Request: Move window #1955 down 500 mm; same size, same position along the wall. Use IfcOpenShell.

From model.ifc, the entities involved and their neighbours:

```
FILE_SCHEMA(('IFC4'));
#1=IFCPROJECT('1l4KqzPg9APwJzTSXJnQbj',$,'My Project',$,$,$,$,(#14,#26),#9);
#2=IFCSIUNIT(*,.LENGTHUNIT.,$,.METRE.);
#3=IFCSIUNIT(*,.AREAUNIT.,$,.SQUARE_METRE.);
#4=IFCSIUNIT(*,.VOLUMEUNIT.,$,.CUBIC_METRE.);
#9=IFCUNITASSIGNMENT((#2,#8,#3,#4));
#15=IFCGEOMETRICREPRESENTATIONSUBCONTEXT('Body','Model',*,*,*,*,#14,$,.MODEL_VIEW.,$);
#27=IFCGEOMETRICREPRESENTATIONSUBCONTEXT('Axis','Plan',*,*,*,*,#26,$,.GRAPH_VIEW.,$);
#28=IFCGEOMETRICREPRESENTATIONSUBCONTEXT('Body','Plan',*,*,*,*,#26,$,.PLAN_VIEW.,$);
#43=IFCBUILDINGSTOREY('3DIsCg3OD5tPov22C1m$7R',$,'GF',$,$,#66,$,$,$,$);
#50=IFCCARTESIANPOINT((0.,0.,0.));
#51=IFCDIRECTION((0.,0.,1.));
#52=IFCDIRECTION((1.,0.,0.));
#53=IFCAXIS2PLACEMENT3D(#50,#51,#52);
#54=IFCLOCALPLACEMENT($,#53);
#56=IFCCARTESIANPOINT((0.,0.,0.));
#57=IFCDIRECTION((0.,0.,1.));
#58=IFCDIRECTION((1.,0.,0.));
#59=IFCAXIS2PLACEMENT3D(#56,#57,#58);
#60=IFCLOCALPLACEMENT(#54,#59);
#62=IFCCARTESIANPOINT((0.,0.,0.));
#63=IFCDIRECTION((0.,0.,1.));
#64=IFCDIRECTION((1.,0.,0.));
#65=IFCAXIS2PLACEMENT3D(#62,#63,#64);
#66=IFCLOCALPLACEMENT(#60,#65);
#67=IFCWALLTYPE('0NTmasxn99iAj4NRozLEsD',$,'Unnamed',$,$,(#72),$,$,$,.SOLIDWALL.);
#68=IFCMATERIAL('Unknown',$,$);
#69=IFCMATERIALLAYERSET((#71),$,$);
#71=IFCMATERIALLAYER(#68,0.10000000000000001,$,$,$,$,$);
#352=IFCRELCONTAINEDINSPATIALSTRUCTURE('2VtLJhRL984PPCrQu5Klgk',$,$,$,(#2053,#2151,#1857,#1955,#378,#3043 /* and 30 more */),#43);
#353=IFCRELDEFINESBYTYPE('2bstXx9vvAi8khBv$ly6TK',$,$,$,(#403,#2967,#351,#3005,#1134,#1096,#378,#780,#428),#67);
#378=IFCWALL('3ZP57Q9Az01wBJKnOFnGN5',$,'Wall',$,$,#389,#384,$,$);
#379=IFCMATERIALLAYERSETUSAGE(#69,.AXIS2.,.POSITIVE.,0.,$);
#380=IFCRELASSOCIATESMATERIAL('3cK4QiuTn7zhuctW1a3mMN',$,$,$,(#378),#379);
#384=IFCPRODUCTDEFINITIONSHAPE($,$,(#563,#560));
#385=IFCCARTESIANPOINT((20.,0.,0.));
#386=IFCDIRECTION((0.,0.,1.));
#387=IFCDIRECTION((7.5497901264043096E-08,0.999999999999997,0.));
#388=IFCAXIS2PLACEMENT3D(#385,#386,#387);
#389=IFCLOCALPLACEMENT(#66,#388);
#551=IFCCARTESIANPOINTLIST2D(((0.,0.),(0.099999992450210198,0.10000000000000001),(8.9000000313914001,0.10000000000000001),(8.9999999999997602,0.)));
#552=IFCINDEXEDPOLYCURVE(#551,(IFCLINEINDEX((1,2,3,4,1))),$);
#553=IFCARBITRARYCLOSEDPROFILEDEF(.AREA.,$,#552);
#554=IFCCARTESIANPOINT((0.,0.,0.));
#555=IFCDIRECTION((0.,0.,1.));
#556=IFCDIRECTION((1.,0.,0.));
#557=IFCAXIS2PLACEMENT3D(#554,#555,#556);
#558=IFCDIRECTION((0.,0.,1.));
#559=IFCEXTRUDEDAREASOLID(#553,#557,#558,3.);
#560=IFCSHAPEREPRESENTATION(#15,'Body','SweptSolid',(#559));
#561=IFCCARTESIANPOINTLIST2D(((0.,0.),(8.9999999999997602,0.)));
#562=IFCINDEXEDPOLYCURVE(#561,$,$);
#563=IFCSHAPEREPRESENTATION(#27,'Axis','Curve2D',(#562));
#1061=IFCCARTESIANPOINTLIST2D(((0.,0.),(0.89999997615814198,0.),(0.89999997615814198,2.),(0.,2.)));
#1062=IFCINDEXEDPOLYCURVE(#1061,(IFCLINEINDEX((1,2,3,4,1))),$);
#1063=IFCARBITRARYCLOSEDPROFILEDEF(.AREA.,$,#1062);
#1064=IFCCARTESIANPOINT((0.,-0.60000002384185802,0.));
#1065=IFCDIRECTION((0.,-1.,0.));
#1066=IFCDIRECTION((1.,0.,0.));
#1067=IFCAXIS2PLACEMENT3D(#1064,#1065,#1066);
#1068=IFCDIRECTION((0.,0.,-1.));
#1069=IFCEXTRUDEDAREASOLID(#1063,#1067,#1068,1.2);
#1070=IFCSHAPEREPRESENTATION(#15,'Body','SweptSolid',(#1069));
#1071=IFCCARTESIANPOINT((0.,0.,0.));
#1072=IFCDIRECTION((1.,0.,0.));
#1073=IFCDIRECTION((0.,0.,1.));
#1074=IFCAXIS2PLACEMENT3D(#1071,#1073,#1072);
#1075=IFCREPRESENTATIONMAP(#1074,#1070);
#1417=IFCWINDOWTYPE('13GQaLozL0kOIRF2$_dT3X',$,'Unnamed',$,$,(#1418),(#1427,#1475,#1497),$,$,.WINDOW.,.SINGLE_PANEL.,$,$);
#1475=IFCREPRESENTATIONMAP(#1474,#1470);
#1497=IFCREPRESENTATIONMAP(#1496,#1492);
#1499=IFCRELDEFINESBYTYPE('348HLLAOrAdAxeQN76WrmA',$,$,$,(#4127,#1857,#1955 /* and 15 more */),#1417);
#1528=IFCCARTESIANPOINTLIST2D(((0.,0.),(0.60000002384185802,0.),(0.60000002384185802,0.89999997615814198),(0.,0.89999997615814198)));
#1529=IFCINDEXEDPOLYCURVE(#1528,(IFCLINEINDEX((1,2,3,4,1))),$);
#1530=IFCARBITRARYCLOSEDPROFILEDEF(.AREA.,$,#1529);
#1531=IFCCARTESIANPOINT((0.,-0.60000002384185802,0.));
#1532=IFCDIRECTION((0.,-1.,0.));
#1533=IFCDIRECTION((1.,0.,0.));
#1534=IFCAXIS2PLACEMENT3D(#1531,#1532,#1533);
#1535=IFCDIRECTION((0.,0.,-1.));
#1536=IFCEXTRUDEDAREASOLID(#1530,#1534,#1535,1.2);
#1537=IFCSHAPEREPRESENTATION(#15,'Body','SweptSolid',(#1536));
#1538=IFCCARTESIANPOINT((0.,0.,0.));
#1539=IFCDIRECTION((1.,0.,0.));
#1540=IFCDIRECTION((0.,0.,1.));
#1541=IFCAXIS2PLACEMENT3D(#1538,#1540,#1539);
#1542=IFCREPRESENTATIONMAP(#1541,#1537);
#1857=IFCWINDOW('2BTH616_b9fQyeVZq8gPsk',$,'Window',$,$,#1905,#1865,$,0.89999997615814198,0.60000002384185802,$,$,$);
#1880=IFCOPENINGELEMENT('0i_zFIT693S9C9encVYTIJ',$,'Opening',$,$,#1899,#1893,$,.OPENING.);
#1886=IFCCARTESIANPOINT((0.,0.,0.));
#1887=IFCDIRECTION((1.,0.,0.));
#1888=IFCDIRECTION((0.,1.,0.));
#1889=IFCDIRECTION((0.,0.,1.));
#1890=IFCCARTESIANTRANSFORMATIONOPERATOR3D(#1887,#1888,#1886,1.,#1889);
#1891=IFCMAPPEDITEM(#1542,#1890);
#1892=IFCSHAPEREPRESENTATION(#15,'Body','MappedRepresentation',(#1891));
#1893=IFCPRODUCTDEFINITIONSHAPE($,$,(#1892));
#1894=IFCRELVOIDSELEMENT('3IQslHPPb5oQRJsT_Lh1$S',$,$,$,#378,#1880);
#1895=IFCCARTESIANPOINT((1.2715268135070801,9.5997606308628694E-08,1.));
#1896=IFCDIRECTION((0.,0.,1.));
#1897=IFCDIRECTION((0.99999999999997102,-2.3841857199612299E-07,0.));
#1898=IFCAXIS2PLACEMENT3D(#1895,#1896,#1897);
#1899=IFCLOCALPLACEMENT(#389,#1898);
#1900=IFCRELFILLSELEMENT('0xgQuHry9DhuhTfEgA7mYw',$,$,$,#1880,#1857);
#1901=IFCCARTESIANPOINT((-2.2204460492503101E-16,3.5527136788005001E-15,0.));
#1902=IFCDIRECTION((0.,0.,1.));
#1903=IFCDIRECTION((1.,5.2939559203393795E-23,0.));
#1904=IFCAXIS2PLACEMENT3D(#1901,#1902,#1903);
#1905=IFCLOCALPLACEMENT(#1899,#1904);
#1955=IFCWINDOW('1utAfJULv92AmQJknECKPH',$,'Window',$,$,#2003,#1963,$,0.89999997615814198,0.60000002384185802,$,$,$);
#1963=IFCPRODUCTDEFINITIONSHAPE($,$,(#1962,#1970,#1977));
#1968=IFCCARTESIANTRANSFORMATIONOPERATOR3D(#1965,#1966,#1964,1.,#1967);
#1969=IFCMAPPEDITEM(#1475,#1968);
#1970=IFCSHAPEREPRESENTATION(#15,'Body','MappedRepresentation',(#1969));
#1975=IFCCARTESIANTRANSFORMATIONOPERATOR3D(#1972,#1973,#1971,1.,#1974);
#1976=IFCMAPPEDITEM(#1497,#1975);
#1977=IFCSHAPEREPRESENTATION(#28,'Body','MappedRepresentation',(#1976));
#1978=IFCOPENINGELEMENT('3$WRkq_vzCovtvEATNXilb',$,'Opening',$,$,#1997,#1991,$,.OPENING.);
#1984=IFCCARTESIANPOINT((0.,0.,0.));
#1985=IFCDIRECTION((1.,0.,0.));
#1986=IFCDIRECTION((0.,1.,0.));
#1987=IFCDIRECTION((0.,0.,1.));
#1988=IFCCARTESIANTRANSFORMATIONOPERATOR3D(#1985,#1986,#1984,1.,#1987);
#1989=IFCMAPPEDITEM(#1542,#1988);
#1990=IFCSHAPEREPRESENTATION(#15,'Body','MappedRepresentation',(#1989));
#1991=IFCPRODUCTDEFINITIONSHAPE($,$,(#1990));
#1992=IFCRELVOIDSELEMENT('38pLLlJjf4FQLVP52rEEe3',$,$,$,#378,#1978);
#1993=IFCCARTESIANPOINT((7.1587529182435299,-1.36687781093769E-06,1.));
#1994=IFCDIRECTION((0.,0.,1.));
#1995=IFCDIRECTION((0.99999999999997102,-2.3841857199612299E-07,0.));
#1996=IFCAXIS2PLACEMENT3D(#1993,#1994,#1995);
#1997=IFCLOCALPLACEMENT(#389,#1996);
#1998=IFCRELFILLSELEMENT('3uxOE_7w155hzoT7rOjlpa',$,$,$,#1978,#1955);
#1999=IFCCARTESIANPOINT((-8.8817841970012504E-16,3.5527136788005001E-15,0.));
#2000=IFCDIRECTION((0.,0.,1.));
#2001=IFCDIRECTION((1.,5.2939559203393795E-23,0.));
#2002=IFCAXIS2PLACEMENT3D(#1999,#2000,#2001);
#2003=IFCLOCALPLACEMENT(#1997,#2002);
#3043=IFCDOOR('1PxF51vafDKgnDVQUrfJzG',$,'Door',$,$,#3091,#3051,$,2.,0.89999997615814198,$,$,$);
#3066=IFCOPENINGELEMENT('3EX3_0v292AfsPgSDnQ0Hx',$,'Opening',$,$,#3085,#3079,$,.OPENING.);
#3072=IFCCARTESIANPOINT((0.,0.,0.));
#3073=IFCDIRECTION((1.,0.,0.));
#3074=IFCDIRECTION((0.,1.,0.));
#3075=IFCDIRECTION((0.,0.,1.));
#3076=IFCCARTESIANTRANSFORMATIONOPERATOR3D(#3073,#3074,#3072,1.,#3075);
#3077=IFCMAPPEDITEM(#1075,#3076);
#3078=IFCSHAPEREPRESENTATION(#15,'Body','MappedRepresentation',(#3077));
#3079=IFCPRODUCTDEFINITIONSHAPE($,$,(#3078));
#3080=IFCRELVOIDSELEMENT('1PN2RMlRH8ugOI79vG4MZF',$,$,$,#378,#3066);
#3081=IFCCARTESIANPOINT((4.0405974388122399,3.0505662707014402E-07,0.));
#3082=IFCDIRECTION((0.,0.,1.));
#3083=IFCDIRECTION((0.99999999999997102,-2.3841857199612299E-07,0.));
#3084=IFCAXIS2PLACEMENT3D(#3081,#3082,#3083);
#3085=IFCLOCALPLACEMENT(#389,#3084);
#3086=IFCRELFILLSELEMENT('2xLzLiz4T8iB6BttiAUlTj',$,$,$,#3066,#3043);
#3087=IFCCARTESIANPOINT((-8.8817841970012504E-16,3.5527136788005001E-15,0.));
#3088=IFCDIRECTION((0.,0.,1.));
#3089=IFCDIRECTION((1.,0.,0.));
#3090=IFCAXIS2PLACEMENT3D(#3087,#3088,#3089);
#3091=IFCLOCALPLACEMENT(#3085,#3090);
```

```python
import numpy as np
import ifcopenshell
import ifcopenshell.api.geometry
import ifcopenshell.util.placement
import ifcopenshell.util.unit

model = ifcopenshell.open("model.ifc")
unit_scale = ifcopenshell.util.unit.calculate_unit_scale(model)

window = model.by_id(1955)
opening = window.FillsVoids[0].RelatingOpeningElement
dz = -0.5

shift = np.array([0.0, 0.0, dz])
# The window is placed relative to its opening, so it follows when the opening moves.
matrix = ifcopenshell.util.placement.get_local_placement(opening.ObjectPlacement)
matrix[:3, 3] += shift
ifcopenshell.api.geometry.edit_object_placement(
    model, product=opening, matrix=matrix, is_si=False, should_transform_children=True
)

print(f"moved by {dz * unit_scale:+.3f} m")

model.write("model_edited.ifc")
```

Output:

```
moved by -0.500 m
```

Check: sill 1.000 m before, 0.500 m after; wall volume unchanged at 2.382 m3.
